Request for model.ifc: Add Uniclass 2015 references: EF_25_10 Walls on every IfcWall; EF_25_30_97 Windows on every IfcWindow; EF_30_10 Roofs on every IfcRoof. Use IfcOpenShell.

First a look at what the model holds.

```python
import ifcopenshell

model = ifcopenshell.open("model.ifc")
print(model.schema)
print("classifications:", [c.Name for c in model.by_type("IfcClassification")])
for ifc_class in ("IfcDoor", "IfcRoof", "IfcStair", "IfcWall", "IfcWindow"):
    print(ifc_class, len(model.by_type(ifc_class)))
```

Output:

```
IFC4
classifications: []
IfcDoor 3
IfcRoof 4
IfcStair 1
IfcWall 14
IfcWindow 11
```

```python
import ifcopenshell
import ifcopenshell.api.classification

model = ifcopenshell.open("model.ifc")

system = ifcopenshell.api.classification.add_classification(model, classification="Uniclass 2015")

codes = {
    "IfcWall": ("EF_25_10", "Walls"),
    "IfcWindow": ("EF_25_30_97", "Windows"),
    "IfcRoof": ("EF_30_10", "Roofs"),
}
for ifc_class, (code, name) in codes.items():
    products = model.by_type(ifc_class)
    ifcopenshell.api.classification.add_reference(
        model, products=products, classification=system, identification=code, name=name
    )
    print(code, len(products))

model.write("model_rev.ifc")
```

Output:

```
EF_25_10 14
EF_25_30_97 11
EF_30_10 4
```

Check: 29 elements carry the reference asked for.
